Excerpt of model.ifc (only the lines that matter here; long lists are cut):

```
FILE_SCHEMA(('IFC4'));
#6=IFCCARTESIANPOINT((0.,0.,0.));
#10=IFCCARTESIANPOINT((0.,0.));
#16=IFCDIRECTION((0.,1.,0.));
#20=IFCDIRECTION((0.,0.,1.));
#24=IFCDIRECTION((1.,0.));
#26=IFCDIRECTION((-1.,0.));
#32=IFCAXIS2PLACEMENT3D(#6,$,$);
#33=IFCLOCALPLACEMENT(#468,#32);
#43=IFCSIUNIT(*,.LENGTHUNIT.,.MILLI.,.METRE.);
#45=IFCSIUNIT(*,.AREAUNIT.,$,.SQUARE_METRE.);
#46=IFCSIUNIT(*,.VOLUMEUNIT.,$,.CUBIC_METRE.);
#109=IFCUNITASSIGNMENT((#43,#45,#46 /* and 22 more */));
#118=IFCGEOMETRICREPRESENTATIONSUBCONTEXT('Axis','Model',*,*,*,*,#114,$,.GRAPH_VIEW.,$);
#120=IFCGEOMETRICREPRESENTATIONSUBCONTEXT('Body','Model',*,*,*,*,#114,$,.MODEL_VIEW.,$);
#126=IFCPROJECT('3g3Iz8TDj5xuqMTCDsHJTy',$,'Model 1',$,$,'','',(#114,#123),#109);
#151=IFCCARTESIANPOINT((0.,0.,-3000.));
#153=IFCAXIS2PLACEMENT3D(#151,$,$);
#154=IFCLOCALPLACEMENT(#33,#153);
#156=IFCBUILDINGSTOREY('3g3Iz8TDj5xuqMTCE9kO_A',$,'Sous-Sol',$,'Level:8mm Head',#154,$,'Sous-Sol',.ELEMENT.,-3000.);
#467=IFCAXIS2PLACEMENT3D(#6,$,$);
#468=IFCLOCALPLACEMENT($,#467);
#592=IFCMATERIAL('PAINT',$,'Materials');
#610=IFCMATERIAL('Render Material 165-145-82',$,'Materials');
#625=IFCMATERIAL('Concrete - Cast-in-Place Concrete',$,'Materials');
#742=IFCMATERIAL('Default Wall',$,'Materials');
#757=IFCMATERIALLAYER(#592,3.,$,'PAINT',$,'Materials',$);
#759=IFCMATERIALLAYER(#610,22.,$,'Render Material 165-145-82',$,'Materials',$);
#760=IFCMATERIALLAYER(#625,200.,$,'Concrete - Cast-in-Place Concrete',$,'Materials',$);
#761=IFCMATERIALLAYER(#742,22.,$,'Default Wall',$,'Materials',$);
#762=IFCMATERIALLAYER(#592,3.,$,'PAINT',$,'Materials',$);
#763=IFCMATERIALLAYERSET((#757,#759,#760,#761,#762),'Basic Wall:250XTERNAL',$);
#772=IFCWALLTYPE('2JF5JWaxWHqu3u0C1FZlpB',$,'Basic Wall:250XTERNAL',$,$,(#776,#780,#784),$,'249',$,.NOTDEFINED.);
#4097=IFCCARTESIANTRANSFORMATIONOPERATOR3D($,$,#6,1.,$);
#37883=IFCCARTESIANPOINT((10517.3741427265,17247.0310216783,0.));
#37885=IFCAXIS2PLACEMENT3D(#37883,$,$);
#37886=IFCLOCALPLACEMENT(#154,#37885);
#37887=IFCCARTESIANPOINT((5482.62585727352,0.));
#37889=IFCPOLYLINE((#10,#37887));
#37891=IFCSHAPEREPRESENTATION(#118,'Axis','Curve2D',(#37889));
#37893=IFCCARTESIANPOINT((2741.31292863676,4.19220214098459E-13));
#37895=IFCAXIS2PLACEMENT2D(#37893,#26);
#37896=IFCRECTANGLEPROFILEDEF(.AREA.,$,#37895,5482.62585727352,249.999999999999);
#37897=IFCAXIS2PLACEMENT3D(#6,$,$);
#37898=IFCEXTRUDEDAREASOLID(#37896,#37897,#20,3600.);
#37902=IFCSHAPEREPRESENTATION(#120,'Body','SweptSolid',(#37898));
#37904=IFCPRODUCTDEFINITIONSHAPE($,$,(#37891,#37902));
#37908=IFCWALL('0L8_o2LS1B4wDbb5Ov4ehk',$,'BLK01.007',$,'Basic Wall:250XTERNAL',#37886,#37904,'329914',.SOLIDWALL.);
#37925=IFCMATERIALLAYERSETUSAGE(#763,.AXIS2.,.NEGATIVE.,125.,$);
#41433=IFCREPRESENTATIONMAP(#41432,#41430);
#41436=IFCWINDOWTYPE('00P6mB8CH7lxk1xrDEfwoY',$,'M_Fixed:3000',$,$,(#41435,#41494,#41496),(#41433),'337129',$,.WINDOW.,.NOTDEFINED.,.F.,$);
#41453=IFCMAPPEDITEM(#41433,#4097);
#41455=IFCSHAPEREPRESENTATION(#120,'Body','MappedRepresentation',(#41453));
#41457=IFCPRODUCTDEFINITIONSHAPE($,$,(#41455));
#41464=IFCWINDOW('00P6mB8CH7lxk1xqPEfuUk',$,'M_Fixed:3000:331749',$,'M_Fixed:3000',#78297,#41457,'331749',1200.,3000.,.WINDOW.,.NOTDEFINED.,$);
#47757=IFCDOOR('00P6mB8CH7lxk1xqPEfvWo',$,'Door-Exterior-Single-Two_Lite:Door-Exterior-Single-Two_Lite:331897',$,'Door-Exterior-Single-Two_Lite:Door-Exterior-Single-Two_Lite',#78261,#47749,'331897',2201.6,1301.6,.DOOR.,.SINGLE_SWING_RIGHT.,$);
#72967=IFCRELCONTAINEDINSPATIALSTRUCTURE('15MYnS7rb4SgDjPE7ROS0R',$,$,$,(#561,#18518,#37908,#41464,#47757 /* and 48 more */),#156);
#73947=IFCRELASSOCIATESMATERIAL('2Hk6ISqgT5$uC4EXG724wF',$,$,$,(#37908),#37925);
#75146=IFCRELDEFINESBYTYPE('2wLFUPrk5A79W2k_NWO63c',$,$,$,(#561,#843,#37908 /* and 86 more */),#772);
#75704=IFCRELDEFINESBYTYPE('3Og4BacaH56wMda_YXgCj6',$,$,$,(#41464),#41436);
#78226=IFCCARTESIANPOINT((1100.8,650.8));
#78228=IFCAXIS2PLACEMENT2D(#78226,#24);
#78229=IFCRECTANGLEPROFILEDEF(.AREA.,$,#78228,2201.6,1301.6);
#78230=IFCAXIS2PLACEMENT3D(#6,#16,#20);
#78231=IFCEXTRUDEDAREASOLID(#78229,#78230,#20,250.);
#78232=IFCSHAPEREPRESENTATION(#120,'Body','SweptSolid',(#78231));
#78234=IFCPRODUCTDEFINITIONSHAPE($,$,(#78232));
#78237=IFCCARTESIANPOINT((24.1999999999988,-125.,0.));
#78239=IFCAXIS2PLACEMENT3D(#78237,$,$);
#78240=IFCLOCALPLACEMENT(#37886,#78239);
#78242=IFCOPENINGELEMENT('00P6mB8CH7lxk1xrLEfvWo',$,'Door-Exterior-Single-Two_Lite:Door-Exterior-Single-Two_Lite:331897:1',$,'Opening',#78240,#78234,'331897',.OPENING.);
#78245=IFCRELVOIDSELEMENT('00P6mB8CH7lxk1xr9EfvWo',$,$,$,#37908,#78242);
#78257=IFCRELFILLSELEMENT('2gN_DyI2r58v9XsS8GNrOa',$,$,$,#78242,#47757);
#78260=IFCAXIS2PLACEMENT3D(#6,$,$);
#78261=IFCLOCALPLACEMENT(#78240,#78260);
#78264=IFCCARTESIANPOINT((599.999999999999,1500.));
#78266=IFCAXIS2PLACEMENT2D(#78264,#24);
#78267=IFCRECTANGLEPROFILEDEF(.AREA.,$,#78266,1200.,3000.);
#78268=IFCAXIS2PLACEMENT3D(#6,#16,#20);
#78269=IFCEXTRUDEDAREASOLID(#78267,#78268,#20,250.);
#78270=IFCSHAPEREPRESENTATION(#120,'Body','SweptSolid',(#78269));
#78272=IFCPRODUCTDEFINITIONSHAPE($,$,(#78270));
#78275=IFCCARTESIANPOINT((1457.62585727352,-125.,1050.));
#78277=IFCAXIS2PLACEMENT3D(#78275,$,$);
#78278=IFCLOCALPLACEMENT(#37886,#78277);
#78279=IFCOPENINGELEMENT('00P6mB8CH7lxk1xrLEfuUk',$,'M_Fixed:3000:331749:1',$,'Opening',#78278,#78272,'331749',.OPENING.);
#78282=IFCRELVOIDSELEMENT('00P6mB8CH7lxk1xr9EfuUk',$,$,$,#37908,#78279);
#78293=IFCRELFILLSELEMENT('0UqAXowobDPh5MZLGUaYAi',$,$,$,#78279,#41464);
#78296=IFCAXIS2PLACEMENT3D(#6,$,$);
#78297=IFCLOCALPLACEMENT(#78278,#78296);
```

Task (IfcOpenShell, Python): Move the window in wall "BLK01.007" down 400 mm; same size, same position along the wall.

```python
import numpy as np
import ifcopenshell
import ifcopenshell.api.geometry
import ifcopenshell.util.placement
import ifcopenshell.util.unit

model = ifcopenshell.open("model.ifc")
unit_scale = ifcopenshell.util.unit.calculate_unit_scale(model)

window = model.by_guid("00P6mB8CH7lxk1xqPEfuUk")
opening = window.FillsVoids[0].RelatingOpeningElement
dz = -400.0

shift = np.array([0.0, 0.0, dz])
# The window is placed relative to its opening, so it follows when the opening moves.
matrix = ifcopenshell.util.placement.get_local_placement(opening.ObjectPlacement)
matrix[:3, 3] += shift
ifcopenshell.api.geometry.edit_object_placement(
    model, product=opening, matrix=matrix, is_si=False, should_transform_children=True
)

print(f"moved by {dz * unit_scale:+.3f} m")

model.write("model-out.ifc")
```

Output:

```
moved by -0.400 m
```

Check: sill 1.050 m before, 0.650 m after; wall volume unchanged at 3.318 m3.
